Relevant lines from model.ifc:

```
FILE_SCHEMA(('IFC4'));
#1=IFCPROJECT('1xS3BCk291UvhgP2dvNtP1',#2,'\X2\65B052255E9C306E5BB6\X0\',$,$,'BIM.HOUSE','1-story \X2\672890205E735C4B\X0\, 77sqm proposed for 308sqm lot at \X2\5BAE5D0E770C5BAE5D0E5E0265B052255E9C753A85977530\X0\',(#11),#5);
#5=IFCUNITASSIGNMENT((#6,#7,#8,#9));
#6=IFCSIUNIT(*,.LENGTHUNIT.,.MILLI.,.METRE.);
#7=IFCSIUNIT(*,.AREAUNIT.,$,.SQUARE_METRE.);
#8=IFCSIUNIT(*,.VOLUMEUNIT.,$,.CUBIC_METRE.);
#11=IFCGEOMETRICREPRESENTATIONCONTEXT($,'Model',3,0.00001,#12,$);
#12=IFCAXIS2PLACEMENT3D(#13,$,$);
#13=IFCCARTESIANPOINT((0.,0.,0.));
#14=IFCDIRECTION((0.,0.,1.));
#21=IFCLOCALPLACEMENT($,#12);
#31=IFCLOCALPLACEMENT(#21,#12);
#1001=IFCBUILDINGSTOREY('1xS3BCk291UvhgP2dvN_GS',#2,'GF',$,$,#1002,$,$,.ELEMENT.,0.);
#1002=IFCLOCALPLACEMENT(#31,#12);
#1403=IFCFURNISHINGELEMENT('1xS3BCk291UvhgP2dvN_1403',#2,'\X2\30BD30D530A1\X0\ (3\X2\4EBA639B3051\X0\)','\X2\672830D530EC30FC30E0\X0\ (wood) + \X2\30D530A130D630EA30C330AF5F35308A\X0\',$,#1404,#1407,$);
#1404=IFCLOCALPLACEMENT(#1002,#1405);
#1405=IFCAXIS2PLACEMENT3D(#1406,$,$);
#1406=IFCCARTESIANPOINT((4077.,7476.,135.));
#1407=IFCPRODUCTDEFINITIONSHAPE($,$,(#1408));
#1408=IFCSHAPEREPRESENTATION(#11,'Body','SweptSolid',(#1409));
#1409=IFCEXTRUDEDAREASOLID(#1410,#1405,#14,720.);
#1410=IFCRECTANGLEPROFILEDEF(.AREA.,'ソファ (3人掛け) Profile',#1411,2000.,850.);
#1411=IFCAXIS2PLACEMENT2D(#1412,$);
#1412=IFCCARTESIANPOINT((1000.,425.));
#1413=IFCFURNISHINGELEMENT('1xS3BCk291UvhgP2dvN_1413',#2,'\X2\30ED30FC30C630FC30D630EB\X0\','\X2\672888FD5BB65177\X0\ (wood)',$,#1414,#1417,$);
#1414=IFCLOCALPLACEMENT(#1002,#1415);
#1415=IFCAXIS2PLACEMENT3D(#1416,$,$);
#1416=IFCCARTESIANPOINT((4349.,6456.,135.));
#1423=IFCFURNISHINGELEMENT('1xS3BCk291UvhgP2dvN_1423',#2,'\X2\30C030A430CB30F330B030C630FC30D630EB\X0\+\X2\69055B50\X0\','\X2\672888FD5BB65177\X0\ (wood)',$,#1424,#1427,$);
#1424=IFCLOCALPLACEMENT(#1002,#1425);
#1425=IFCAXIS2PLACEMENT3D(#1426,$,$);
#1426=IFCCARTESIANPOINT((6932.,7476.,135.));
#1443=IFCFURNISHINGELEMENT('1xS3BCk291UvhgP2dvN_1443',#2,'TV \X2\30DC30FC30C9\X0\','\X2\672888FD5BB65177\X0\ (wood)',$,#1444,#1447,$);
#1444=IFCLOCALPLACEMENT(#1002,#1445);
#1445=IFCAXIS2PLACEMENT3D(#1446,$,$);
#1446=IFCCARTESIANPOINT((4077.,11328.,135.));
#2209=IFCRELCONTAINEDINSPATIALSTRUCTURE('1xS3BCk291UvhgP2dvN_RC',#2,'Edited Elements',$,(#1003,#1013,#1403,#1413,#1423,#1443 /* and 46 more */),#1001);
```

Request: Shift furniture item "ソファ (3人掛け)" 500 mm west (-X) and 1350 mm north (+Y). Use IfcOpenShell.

```python
import ifcopenshell
import ifcopenshell.api.geometry
import ifcopenshell.util.placement
import ifcopenshell.util.unit

model = ifcopenshell.open("model.ifc")
unit_scale = ifcopenshell.util.unit.calculate_unit_scale(model)

item = model.by_guid("1xS3BCk291UvhgP2dvN_1403")
matrix = ifcopenshell.util.placement.get_local_placement(item.ObjectPlacement)
matrix[0, 3] -= 0.5 / unit_scale
matrix[1, 3] += 1.35 / unit_scale
ifcopenshell.api.geometry.edit_object_placement(model, product=item, matrix=matrix, is_si=False)

print(ifcopenshell.util.placement.get_local_placement(item.ObjectPlacement).round(3) + 0.0)

model.write("model_updated.ifc")
```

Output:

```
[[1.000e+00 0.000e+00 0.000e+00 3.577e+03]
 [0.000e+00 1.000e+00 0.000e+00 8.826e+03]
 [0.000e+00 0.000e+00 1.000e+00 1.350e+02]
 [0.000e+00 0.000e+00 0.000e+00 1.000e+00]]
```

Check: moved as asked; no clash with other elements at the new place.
